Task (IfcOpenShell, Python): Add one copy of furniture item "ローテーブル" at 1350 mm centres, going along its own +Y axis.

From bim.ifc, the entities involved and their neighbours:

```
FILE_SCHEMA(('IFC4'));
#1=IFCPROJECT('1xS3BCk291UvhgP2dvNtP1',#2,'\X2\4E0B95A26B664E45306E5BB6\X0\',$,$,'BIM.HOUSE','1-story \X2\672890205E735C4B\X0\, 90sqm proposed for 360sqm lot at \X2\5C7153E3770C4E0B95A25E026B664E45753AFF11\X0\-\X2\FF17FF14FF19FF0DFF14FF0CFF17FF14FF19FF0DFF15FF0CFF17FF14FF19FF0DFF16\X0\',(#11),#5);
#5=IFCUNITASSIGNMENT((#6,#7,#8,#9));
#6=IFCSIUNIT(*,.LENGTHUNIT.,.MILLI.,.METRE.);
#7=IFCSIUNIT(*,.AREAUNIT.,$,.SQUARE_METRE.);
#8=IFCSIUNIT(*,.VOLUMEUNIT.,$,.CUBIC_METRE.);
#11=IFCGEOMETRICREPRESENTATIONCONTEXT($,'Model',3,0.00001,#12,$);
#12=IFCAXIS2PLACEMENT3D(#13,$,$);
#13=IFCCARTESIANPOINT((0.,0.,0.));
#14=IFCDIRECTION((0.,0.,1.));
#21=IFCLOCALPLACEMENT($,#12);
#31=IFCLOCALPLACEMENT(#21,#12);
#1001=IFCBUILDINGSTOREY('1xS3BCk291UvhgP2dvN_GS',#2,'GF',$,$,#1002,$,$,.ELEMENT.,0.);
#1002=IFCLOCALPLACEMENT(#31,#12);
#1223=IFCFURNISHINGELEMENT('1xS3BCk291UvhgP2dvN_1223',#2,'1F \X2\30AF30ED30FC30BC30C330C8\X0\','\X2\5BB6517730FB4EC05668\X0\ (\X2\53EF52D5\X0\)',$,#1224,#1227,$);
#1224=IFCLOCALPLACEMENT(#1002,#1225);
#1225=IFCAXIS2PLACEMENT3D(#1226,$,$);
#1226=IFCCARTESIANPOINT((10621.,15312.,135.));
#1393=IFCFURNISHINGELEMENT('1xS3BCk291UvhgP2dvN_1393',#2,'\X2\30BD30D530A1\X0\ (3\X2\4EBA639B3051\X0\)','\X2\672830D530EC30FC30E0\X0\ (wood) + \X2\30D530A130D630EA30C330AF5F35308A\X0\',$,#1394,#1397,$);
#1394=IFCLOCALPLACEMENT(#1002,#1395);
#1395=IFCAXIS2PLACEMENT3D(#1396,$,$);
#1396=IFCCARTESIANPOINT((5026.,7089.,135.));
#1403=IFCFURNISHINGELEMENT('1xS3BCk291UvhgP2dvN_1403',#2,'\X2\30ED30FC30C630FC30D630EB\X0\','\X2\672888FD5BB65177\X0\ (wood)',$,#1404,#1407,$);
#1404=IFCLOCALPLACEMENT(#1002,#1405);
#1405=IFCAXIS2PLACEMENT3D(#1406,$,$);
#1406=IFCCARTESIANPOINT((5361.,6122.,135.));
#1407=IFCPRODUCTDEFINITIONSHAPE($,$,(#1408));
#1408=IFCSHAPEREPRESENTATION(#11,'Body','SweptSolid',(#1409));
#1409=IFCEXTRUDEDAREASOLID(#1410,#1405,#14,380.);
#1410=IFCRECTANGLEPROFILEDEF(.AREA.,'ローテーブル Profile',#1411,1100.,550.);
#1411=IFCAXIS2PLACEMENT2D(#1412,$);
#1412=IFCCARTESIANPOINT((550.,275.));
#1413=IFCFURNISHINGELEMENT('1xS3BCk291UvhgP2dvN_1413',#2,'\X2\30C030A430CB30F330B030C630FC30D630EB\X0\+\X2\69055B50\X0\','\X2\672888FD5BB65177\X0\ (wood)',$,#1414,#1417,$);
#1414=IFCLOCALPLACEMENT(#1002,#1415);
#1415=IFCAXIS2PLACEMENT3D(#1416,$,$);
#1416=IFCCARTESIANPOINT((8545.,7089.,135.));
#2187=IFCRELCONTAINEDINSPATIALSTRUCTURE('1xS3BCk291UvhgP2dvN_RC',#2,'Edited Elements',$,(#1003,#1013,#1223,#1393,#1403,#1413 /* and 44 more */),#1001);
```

```python
import ifcopenshell
import ifcopenshell.api.geometry
import ifcopenshell.api.root
import ifcopenshell.util.element
import ifcopenshell.util.placement

model = ifcopenshell.open("bim.ifc")


def reuse_history(source, copy):
    """copy_class also copies each property set's owner history, people and application; keep the originals."""
    for rel in copy.IsDefinedBy:
        if rel.is_a("IfcRelDefinesByProperties") and (history := rel.RelatingPropertyDefinition.OwnerHistory):
            rel.RelatingPropertyDefinition.OwnerHistory = source.OwnerHistory
            ifcopenshell.util.element.remove_deep2(model, history)


source = model.by_guid("1xS3BCk291UvhgP2dvN_1403")
base = ifcopenshell.util.placement.get_local_placement(source.ObjectPlacement)
step = base[:3, 1] * 1350.0

for i in range(1, 2):
    copy = ifcopenshell.api.root.copy_class(model, product=source)
    copy.Representation = ifcopenshell.util.element.copy_deep(
        model, source.Representation, exclude=["IfcGeometricRepresentationContext", "IfcRepresentationMap"]
    )
    reuse_history(source, copy)
    matrix = base.copy()
    matrix[:3, 3] += i * step
    print("added at", matrix[:3, 3].round(3) + 0.0)
    ifcopenshell.api.geometry.edit_object_placement(model, product=copy, matrix=matrix, is_si=False)

model.write("bim_updated.ifc")
```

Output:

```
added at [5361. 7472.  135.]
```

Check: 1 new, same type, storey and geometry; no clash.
